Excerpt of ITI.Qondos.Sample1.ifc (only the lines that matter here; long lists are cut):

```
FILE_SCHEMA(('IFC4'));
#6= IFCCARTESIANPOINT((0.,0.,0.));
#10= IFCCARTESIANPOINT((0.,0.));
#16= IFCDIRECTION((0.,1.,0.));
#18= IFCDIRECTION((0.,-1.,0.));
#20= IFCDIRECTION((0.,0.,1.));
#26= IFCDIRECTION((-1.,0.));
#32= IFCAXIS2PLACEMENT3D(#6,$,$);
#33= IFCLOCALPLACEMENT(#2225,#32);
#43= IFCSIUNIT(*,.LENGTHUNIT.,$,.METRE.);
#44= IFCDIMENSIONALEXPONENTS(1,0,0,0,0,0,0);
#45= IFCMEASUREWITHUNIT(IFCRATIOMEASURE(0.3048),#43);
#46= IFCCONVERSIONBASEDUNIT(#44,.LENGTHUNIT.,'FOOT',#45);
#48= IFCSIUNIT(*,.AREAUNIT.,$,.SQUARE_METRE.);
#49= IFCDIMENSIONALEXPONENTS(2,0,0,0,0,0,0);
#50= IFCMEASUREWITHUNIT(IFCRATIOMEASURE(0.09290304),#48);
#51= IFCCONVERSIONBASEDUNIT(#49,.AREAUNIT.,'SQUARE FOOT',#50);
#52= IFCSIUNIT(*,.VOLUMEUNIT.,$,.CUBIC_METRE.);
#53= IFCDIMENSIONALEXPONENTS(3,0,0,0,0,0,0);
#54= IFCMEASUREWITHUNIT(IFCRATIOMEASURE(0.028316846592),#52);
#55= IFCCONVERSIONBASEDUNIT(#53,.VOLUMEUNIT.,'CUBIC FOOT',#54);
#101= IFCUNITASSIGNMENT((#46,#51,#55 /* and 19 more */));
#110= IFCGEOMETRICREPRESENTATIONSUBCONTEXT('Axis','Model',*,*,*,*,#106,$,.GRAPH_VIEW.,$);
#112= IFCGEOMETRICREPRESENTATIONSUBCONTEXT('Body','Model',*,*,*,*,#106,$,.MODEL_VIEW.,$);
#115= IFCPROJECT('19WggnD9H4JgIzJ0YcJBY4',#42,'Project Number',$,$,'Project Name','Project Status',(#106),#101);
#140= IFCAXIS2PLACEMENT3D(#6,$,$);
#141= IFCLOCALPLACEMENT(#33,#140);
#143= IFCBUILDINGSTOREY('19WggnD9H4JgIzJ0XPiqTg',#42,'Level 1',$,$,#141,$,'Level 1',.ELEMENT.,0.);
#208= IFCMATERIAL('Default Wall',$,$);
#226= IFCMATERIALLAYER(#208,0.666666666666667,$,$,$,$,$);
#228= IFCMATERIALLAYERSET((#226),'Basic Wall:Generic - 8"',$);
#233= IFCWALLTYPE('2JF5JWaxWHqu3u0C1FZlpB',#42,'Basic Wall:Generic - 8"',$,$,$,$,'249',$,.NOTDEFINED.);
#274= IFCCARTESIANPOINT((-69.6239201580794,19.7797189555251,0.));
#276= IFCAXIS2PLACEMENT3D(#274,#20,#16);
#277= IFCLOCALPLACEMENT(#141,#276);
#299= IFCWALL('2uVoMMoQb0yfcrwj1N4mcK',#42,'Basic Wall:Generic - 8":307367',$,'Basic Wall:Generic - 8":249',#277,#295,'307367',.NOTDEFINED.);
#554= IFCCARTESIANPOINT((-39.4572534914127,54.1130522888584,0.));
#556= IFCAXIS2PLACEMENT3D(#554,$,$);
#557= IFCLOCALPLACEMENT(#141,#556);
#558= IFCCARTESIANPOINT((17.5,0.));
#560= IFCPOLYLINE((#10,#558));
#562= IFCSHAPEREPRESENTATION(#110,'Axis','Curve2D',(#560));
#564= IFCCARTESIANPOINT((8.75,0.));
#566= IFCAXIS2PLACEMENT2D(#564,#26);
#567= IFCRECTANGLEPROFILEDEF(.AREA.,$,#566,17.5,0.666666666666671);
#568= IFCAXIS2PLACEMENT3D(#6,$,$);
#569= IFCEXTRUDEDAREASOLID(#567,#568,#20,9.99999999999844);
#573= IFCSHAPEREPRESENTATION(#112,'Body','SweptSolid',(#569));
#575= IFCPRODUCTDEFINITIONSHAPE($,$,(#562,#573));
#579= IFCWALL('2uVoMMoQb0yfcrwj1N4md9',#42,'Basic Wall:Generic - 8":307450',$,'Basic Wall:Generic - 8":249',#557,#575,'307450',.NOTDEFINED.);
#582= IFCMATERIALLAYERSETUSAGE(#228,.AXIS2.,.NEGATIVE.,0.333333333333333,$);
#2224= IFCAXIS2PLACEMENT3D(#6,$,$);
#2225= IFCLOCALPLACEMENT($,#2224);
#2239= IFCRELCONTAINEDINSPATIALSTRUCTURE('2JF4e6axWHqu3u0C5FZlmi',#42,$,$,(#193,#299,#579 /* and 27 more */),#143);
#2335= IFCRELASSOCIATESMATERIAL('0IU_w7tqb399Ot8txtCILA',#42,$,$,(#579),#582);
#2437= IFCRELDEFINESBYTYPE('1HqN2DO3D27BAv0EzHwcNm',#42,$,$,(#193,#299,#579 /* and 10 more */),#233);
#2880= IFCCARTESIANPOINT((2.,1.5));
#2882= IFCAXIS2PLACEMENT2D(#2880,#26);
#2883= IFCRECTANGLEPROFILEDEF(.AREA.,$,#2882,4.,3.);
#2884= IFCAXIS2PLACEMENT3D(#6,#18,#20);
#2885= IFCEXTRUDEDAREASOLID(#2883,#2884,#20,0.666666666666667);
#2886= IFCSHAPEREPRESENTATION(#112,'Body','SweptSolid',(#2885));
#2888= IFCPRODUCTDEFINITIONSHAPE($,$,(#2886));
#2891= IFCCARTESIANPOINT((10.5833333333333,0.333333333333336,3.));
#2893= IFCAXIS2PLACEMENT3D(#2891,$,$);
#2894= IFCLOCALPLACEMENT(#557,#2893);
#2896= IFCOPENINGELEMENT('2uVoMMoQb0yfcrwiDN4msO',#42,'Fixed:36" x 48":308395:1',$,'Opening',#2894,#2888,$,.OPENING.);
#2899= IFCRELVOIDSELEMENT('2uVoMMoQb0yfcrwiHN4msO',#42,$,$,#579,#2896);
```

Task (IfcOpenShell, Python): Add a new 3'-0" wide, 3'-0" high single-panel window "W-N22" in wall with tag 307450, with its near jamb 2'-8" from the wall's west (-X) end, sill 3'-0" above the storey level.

```python
import numpy as np
import ifcopenshell
import ifcopenshell.api.feature
import ifcopenshell.api.geometry
import ifcopenshell.api.root
import ifcopenshell.api.spatial
import ifcopenshell.geom
import ifcopenshell.util.element
import ifcopenshell.util.placement
import ifcopenshell.util.representation
import ifcopenshell.util.shape
import ifcopenshell.util.unit

model = ifcopenshell.open("ITI.Qondos.Sample1.ifc")
unit_scale = ifcopenshell.util.unit.calculate_unit_scale(model)
settings = ifcopenshell.geom.settings()


def volume(element):
    """Net volume in cubic metres, openings subtracted."""
    shape = ifcopenshell.geom.create_shape(settings, element)
    return ifcopenshell.util.shape.get_volume(shape.geometry)


wall = model.by_guid("2uVoMMoQb0yfcrwj1N4md9")
storey = ifcopenshell.util.element.get_container(wall, ifc_class="IfcBuildingStorey")
context = ifcopenshell.util.representation.get_context(model, "Model", "Body", "MODEL_VIEW")
before = volume(wall)

width, height, from_end, sill = 0.9144, 0.9144, 0.8128, 0.9144  # metres

# The wall runs along its own X axis, and the end named is its -X end.
wall_shape = ifcopenshell.geom.create_shape(settings, wall)
x, y, z = ifcopenshell.util.shape.get_vertices(wall_shape.geometry).T
start = x.min() + from_end
face, thickness = float(y.min()), float(y.max() - y.min())
wall_matrix = ifcopenshell.util.placement.get_local_placement(wall.ObjectPlacement)
level = ifcopenshell.util.placement.get_local_placement(storey.ObjectPlacement)[2, 3]


def in_wall(x, y):
    """Placement at x, y metres in the wall's axes, at sill height."""
    matrix = wall_matrix.copy()
    matrix[:, 3] = wall_matrix @ np.array([x / unit_scale, y / unit_scale, 0.0, 1.0])
    matrix[2, 3] = level + sill / unit_scale
    return matrix


# Opening: a box that overshoots both wall faces by 50 mm.
opening = ifcopenshell.api.root.create_entity(model, ifc_class="IfcOpeningElement", predefined_type="OPENING")
box = ifcopenshell.api.geometry.add_wall_representation(
    model, context=context, length=width, height=height, thickness=thickness + 0.1
)
ifcopenshell.api.geometry.assign_representation(model, product=opening, representation=box)
ifcopenshell.api.geometry.edit_object_placement(model, product=opening, matrix=in_wall(start, face - 0.05), is_si=False)
ifcopenshell.api.feature.add_feature(model, feature=opening, element=wall)

window = ifcopenshell.api.root.create_entity(model, ifc_class="IfcWindow", name="W-N22", predefined_type="WINDOW")
window.OverallWidth, window.OverallHeight = width / unit_scale, height / unit_scale
window.PartitioningType = "SINGLE_PANEL"
body = ifcopenshell.api.geometry.add_window_representation(
    model,
    context=context,
    overall_width=window.OverallWidth,
    overall_height=window.OverallHeight,
    partition_type="SINGLE_PANEL",
)
ifcopenshell.api.geometry.assign_representation(model, product=window, representation=body)
ifcopenshell.api.spatial.assign_container(model, products=[window], relating_structure=storey)
ifcopenshell.api.feature.add_filling(model, opening=opening, element=window)

# Centre the window in the wall's thickness.
ifcopenshell.api.geometry.edit_object_placement(model, product=window, matrix=in_wall(start, face), is_si=False)
window_shape = ifcopenshell.geom.create_shape(settings, window)
depth = ifcopenshell.util.shape.get_vertices(window_shape.geometry)[:, 1]
offset = face + thickness / 2 - (depth.min() + depth.max()) / 2
ifcopenshell.api.geometry.edit_object_placement(model, product=window, matrix=in_wall(start, offset), is_si=False)

after = volume(wall)

print(f"wall volume {before:.3f} -> {after:.3f} m3")

model.write("ITI.Qondos.Sample1_edited.ifc")
```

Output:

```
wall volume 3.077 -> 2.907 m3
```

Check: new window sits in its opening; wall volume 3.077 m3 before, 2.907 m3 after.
